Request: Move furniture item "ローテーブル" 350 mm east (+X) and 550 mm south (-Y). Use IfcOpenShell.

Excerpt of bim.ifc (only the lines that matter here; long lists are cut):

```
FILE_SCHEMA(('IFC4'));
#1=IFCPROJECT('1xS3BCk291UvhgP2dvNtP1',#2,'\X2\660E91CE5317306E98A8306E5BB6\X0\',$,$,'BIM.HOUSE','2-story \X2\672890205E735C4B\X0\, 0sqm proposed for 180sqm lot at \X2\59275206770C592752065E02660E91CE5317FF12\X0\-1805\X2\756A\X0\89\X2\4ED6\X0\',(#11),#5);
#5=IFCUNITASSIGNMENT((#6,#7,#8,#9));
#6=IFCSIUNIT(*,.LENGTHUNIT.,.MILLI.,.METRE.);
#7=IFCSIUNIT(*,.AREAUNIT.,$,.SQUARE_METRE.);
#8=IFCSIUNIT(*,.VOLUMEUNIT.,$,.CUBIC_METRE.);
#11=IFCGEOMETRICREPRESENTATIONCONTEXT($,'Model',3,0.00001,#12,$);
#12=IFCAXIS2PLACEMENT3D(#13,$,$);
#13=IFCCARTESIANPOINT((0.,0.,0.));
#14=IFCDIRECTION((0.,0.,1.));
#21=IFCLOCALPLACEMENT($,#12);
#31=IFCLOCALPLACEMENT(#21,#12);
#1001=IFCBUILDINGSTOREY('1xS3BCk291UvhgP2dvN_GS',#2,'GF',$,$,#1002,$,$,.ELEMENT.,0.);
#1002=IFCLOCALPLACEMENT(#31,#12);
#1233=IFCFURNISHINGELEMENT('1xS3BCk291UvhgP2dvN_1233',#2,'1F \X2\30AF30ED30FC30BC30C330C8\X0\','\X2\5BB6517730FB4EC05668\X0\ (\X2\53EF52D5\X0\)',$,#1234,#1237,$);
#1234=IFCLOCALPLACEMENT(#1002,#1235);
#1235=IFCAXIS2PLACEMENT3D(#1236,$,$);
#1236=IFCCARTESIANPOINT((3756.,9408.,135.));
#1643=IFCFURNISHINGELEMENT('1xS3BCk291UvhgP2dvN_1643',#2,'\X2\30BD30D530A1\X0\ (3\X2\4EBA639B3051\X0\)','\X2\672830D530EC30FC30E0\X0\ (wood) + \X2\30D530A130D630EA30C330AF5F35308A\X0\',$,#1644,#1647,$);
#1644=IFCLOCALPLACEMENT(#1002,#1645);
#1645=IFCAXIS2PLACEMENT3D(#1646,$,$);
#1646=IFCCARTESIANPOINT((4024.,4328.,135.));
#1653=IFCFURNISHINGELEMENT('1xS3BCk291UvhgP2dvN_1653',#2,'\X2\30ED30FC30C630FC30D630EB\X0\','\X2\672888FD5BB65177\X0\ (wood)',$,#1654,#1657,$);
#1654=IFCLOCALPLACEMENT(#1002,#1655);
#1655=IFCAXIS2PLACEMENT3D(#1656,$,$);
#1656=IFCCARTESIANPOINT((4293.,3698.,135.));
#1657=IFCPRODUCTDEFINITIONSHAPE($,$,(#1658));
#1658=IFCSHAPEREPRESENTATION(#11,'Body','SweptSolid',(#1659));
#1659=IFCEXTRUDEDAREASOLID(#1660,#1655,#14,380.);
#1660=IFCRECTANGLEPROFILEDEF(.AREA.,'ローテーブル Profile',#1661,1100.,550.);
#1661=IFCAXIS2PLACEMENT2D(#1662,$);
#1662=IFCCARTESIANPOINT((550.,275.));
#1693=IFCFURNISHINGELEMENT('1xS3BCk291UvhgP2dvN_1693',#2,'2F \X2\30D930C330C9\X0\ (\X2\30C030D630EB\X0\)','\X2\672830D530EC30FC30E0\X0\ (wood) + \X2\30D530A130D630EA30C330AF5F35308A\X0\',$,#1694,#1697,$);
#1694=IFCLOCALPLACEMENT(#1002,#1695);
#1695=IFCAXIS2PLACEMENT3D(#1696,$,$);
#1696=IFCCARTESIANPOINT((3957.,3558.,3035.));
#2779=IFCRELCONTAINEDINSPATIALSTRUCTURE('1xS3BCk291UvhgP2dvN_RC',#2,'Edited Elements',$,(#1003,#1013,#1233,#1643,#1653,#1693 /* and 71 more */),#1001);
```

```python
import ifcopenshell
import ifcopenshell.api.geometry
import ifcopenshell.util.placement
import ifcopenshell.util.unit

model = ifcopenshell.open("bim.ifc")
unit_scale = ifcopenshell.util.unit.calculate_unit_scale(model)

item = model.by_id(1653)
matrix = ifcopenshell.util.placement.get_local_placement(item.ObjectPlacement)
matrix[0, 3] += 0.35 / unit_scale
matrix[1, 3] -= 0.55 / unit_scale
ifcopenshell.api.geometry.edit_object_placement(model, product=item, matrix=matrix, is_si=False)

print(ifcopenshell.util.placement.get_local_placement(item.ObjectPlacement).round(3) + 0.0)

model.write("bim_updated.ifc")
```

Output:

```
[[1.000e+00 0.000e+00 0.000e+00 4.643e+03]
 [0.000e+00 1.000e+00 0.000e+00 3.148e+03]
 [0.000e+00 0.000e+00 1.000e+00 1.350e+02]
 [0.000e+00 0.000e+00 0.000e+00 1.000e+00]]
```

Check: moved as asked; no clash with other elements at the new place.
